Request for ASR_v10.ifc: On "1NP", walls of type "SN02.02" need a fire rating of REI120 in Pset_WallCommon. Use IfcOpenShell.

First a look at what the model holds.

```python
import ifcopenshell
import ifcopenshell.util.element

model = ifcopenshell.open("ASR_v10.ifc")
print(model.schema)
storey = next(s for s in model.by_type("IfcBuildingStorey") if s.Name == "1NP")
walls = [e for e in ifcopenshell.util.element.get_decomposition(storey) if e.is_a("IfcWall")]
seen = {}
for e in walls:
    element_type = ifcopenshell.util.element.get_type(e)
    key = (element_type.Name if element_type != e and element_type else None, ifcopenshell.util.element.get_pset(e, "Pset_WallCommon", "FireRating"))
    seen[key] = seen.get(key, 0) + 1
for (name, value), count in sorted(seen.items(), key=str):
    print(count, "x", name, "|", value)
```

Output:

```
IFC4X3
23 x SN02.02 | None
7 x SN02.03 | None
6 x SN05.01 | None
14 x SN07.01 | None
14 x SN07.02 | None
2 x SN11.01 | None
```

```python
import ifcopenshell
import ifcopenshell.api.pset
import ifcopenshell.util.element

model = ifcopenshell.open("ASR_v10.ifc")

storey = next(s for s in model.by_type("IfcBuildingStorey") if s.Name == "1NP")
walls = [e for e in ifcopenshell.util.element.get_decomposition(storey) if e.is_a("IfcWall")]

count = 0
for e in walls:
    element_type = ifcopenshell.util.element.get_type(e)
    if element_type in (None, e) or element_type.Name != "SN02.02":
        continue
    # add_pset returns the element's existing set when there is one.
    pset = ifcopenshell.api.pset.add_pset(model, product=e, name="Pset_WallCommon")
    ifcopenshell.api.pset.edit_pset(model, pset=pset, properties={"FireRating": "REI120"})
    count += 1

print(count, "walls updated")

model.write("ASR_v10_v2.ifc")
```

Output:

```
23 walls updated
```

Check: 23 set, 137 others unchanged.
